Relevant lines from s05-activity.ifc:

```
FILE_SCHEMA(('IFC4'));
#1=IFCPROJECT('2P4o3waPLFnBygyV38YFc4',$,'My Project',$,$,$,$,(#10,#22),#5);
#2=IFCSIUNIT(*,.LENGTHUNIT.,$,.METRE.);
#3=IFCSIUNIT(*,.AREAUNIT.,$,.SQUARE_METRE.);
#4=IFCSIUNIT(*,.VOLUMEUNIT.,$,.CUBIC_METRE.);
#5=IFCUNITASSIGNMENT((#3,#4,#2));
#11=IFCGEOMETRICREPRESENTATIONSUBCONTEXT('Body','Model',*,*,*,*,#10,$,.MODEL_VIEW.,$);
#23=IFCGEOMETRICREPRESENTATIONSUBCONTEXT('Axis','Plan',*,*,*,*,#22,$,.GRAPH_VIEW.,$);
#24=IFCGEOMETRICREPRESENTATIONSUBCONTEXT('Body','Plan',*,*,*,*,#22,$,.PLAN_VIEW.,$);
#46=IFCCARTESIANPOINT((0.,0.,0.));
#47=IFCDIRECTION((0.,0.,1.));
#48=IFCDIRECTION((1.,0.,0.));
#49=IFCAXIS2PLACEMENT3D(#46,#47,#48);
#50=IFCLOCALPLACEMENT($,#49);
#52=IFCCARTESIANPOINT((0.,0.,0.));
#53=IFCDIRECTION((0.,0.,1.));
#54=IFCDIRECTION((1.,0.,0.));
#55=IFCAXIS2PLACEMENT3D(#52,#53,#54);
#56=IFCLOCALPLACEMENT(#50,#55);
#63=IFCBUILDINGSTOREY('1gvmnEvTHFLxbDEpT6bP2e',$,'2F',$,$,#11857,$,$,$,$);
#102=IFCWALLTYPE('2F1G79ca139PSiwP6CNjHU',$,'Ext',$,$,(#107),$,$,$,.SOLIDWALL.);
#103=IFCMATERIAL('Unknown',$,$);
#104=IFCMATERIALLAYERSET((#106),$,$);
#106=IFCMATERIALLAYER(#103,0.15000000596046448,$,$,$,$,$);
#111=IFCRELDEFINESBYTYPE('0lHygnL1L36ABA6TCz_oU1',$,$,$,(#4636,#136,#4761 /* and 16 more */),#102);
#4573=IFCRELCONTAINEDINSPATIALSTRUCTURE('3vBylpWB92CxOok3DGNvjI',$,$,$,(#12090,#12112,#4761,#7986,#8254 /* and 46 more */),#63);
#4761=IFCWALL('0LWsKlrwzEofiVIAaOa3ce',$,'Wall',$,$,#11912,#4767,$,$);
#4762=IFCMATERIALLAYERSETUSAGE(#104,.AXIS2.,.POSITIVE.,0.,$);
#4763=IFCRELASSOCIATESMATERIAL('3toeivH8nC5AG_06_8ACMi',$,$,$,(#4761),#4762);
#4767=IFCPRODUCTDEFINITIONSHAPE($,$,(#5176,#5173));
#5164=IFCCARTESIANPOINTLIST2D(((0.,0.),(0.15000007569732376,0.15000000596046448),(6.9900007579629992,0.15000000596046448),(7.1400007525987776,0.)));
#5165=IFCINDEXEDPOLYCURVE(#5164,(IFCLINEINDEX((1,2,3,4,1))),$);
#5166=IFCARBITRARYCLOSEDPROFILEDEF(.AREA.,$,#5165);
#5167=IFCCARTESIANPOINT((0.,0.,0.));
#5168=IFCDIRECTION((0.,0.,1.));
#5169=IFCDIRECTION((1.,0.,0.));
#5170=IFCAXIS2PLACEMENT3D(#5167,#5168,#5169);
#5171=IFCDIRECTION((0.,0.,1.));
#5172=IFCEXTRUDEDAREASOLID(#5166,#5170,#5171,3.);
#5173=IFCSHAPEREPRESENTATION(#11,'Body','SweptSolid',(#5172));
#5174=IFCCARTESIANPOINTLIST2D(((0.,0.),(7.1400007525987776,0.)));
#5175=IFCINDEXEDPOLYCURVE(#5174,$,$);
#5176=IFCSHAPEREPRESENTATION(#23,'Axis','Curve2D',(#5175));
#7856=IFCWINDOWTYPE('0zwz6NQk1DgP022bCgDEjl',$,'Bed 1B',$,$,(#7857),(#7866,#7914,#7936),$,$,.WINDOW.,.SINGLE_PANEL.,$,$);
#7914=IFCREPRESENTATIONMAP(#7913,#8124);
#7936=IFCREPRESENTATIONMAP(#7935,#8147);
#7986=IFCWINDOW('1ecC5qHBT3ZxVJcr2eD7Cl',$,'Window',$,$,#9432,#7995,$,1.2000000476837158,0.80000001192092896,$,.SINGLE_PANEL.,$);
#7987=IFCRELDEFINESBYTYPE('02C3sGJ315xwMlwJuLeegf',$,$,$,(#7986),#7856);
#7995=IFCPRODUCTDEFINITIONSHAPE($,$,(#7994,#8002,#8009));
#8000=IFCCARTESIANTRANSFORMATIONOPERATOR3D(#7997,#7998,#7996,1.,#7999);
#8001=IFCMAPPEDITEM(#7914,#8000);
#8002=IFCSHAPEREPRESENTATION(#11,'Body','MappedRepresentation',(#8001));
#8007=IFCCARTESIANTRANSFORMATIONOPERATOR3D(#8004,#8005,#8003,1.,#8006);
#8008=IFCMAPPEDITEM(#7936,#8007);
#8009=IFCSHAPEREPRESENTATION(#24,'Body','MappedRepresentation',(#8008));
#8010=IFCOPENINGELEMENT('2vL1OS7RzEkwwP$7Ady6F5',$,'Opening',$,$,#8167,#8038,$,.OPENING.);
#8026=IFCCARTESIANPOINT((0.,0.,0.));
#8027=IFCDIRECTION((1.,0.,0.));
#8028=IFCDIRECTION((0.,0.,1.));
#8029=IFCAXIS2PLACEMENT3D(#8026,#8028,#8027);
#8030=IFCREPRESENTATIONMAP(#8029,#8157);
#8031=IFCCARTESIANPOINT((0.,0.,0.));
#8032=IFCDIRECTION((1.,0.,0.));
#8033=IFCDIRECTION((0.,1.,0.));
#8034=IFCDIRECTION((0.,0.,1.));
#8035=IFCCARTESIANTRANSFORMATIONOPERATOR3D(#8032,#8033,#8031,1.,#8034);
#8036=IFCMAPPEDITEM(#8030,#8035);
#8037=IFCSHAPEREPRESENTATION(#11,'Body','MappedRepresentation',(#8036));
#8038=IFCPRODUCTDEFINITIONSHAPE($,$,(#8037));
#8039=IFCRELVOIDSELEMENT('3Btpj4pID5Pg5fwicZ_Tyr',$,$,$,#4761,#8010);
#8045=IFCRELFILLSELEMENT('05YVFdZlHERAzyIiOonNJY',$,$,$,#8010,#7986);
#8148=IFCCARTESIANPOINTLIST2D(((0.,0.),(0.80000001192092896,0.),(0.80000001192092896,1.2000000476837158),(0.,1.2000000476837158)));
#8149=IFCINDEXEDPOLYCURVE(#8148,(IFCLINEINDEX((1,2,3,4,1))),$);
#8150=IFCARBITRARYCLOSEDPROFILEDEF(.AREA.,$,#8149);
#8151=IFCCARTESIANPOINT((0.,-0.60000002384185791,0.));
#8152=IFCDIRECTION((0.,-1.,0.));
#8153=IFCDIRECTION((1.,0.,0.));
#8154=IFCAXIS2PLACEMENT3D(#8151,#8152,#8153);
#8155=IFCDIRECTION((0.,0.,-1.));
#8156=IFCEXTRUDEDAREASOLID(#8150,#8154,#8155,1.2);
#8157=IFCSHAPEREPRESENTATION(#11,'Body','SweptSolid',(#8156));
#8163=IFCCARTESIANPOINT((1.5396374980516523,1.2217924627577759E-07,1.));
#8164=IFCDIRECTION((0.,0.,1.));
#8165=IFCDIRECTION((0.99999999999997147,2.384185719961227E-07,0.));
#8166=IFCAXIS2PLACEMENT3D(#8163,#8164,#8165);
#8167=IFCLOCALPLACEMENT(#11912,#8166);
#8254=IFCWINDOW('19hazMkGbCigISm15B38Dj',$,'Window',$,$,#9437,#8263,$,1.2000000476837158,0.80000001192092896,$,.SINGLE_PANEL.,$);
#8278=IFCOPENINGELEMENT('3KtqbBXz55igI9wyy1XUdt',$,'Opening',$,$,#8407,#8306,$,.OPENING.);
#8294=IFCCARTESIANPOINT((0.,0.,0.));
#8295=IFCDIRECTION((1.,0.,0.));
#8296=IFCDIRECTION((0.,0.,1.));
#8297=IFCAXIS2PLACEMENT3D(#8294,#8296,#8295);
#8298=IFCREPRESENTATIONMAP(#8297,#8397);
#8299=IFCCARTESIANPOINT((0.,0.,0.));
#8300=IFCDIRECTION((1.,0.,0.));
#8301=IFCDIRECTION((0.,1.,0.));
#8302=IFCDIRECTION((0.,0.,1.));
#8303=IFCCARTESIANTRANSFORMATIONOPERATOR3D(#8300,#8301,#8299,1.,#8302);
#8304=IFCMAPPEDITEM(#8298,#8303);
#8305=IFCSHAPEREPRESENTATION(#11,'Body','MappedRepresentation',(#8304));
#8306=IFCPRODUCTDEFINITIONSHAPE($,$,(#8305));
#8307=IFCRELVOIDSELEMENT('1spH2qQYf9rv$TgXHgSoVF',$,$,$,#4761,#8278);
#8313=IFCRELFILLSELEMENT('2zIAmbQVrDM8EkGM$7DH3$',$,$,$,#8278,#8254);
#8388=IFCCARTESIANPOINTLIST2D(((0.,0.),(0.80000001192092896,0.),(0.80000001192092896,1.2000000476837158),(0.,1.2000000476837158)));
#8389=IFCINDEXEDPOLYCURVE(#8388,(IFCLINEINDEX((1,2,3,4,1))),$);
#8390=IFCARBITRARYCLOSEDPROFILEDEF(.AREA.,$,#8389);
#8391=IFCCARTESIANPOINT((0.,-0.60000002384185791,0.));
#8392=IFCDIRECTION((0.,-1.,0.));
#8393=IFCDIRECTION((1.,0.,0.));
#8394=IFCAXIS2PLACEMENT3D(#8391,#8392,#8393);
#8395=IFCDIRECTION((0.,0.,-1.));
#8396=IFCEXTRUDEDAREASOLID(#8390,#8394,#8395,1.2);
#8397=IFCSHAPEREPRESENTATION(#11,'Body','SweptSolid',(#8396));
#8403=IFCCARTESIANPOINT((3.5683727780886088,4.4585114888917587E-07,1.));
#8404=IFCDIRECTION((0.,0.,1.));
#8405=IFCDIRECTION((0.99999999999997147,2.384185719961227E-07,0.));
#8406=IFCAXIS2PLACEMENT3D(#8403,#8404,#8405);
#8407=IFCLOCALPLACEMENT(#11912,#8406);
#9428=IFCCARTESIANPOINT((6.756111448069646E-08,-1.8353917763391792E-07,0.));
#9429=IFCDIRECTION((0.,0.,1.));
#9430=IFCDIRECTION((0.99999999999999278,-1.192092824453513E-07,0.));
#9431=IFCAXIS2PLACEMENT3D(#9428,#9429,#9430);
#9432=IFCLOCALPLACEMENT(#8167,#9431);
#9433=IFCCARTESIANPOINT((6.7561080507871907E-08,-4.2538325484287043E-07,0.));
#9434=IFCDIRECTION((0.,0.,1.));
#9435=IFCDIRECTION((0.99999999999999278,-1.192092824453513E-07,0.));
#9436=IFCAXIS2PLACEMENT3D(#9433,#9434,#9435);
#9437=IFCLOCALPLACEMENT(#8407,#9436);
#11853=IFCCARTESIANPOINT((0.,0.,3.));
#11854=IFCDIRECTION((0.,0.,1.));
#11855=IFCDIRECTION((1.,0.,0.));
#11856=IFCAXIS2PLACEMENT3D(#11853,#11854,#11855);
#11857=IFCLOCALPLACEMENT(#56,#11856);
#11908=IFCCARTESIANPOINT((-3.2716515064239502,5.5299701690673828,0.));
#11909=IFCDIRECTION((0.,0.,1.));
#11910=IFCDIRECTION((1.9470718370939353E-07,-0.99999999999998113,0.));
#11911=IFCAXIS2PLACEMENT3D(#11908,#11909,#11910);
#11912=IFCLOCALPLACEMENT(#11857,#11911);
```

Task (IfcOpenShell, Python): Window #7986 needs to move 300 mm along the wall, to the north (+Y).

```python
import ifcopenshell
import ifcopenshell.api.geometry
import ifcopenshell.util.placement

model = ifcopenshell.open("s05-activity.ifc")

window = model.by_guid("1ecC5qHBT3ZxVJcr2eD7Cl")
opening = window.FillsVoids[0].RelatingOpeningElement
wall = opening.VoidsElements[0].RelatingBuildingElement

wall_matrix = ifcopenshell.util.placement.get_local_placement(wall.ObjectPlacement)
shift = wall_matrix[:3, 0] * -0.3
before = ifcopenshell.util.placement.get_local_placement(window.ObjectPlacement)[:3, 3].copy()

# The window is placed relative to its opening, so it follows when the opening moves.
matrix = ifcopenshell.util.placement.get_local_placement(opening.ObjectPlacement)
matrix[:3, 3] += shift
ifcopenshell.api.geometry.edit_object_placement(
    model, product=opening, matrix=matrix, is_si=False, should_transform_children=True
)

after = ifcopenshell.util.placement.get_local_placement(window.ObjectPlacement)[:3, 3]
print("window moved by", (after - before).round(3) + 0.0)

model.write("s05-activity_edited.ifc")
```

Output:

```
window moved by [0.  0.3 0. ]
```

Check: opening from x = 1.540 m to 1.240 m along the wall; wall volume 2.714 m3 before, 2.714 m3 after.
